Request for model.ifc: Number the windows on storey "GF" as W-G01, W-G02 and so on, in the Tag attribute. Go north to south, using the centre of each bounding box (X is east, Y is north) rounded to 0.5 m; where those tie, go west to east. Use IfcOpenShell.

First a look at what the model holds.

```python
import ifcopenshell
import ifcopenshell.util.element
import ifcopenshell.util.placement

model = ifcopenshell.open("model.ifc")
print(model.schema)
storey = next(s for s in model.by_type("IfcBuildingStorey") if s.Name == "GF")
windows = [e for e in ifcopenshell.util.element.get_decomposition(storey) if e.is_a("IfcWindow")]
for e in sorted(windows, key=lambda e: e.id()):
    origin = ifcopenshell.util.placement.get_local_placement(e.ObjectPlacement)[:3, 3]
    print(e.id(), e.Tag, e.Name, origin.round(2) + 0.0, sep=" | ")
```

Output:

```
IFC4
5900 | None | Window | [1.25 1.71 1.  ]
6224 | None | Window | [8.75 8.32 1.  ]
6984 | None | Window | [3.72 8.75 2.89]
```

```python
import ifcopenshell
import ifcopenshell.geom
import ifcopenshell.util.element
import ifcopenshell.util.shape

model = ifcopenshell.open("model.ifc")
settings = ifcopenshell.geom.settings()
settings.set("use-world-coords", True)


def centre(element):
    shape = ifcopenshell.geom.create_shape(settings, element)
    return ifcopenshell.util.shape.get_bbox_centroid(shape.geometry)


storey = next(s for s in model.by_type("IfcBuildingStorey") if s.Name == "GF")
windows = [e for e in ifcopenshell.util.element.get_decomposition(storey) if e.is_a("IfcWindow")]

# Insertion points can sit at a corner or the storey origin, so sort by the geometry (in metres).
centres = {e: centre(e) for e in windows}
windows.sort(key=lambda e: (-round(centres[e][1] / 0.5), centres[e][0]))

for i, e in enumerate(windows, start=1):
    number = f"W-G{i:02d}"
    e.Tag = number
    print(e.id(), number)

model.write("model_rev.ifc")
```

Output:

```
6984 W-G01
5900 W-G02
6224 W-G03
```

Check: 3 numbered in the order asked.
